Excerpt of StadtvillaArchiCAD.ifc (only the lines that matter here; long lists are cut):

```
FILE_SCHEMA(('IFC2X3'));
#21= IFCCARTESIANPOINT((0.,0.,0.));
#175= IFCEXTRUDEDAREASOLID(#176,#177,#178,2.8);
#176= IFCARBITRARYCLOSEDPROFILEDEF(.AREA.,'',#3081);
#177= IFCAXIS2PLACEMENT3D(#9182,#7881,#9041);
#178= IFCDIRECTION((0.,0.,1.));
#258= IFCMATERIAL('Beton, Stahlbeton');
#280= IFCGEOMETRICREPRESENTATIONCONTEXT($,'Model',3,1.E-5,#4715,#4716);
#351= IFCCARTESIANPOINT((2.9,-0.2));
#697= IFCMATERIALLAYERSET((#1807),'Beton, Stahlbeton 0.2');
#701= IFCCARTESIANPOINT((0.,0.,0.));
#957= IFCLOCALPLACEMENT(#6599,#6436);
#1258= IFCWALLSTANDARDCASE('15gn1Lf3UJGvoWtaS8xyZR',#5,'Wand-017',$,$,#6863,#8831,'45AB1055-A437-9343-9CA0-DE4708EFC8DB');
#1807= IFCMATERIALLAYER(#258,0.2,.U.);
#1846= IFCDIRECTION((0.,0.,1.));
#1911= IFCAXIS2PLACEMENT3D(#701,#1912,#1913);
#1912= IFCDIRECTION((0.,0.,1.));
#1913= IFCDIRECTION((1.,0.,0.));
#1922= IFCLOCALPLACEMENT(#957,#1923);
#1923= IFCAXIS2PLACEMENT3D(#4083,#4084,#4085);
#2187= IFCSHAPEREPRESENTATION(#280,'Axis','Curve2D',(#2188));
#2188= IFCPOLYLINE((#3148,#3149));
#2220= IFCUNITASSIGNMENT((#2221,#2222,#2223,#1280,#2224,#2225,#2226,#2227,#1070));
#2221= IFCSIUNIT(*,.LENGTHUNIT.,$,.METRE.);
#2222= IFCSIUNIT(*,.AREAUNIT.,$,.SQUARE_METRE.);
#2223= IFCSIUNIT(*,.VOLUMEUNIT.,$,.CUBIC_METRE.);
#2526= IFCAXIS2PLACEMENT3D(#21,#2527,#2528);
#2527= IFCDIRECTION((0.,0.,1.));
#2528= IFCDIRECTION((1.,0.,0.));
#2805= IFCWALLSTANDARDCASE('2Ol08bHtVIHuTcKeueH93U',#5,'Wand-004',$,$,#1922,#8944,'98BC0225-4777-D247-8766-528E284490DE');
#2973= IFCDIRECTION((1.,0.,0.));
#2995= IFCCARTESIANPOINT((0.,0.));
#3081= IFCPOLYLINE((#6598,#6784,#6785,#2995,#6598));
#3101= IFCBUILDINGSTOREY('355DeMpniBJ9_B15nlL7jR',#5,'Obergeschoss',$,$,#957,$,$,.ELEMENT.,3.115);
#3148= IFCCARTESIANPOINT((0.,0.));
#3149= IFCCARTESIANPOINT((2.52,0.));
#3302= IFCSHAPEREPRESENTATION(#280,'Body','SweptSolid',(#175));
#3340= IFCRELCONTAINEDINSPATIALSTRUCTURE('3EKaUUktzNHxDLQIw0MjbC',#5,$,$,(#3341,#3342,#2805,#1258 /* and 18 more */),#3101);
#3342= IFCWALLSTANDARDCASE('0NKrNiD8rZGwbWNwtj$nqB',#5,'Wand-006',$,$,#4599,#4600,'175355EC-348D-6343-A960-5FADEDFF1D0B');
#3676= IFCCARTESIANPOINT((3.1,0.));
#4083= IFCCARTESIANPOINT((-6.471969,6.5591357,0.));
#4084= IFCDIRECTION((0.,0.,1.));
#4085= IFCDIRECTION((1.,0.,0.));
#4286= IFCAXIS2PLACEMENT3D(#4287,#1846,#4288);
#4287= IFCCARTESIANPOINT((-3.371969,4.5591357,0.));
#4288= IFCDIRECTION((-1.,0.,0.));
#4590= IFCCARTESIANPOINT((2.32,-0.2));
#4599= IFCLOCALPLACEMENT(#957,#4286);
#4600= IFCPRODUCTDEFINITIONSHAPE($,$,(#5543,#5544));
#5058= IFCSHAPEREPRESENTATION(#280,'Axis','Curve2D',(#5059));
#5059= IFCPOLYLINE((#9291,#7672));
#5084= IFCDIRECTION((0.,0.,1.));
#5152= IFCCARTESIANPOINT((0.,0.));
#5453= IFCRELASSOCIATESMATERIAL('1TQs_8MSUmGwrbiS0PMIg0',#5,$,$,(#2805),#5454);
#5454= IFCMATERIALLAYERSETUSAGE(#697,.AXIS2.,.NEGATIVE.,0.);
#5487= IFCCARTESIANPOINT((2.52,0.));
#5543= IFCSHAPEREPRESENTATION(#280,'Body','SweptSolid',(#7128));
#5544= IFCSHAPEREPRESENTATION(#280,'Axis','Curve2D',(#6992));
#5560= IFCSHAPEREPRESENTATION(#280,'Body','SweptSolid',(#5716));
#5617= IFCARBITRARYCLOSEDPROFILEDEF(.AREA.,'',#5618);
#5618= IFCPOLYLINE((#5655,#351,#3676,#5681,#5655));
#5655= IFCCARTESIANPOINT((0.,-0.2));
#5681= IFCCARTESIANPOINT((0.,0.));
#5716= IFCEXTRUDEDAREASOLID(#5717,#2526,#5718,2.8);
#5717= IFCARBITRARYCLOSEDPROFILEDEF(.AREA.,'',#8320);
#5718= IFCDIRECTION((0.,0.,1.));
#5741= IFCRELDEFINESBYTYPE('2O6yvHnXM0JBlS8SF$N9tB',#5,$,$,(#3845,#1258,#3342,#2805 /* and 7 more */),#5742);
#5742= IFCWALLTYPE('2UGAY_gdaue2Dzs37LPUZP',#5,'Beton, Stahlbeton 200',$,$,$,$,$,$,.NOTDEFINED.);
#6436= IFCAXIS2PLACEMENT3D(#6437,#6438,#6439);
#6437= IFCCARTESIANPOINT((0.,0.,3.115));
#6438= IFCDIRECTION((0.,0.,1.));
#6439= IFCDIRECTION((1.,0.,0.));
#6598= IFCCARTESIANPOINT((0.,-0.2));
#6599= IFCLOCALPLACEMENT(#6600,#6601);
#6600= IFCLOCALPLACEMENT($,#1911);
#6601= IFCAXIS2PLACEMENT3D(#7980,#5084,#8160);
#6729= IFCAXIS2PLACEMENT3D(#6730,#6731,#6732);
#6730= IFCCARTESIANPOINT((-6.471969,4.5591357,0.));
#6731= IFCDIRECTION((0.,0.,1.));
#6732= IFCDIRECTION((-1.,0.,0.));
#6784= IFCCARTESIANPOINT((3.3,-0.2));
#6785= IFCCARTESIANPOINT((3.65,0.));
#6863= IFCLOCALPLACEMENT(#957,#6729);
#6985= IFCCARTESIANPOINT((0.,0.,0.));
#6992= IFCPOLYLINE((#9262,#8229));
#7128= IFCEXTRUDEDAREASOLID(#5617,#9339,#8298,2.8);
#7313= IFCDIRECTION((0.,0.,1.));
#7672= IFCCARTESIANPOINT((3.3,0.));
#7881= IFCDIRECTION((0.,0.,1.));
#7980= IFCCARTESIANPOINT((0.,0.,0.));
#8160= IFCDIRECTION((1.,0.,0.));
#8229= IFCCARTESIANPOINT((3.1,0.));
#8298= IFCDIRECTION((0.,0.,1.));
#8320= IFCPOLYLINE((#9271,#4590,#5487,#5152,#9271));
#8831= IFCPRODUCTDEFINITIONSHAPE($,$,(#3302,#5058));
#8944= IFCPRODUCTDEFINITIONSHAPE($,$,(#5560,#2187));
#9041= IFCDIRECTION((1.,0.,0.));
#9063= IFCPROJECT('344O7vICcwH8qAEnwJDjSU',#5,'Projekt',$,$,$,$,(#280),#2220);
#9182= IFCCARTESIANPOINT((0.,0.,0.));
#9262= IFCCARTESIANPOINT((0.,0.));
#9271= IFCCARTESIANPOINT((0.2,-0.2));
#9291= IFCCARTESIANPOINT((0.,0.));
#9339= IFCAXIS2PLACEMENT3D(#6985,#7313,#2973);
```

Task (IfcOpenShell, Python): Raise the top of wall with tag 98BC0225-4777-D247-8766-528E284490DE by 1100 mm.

```python
import ifcopenshell
import ifcopenshell.geom
import ifcopenshell.util.shape

model = ifcopenshell.open("StadtvillaArchiCAD.ifc")
settings = ifcopenshell.geom.settings()


def volume(element):
    """Net volume in cubic metres, openings subtracted."""
    shape = ifcopenshell.geom.create_shape(settings, element)
    return ifcopenshell.util.shape.get_volume(shape.geometry)


wall = model.by_id(2805)
before = volume(wall)

body = next(r for r in wall.Representation.Representations if r.RepresentationIdentifier == "Body")
solid = body.Items[0]
old_height = solid.Depth
solid.Depth += 1.1
after = volume(wall)

print(f"height {old_height:g} -> {solid.Depth:g}, volume {before:.3f} -> {after:.3f} m3")

model.write("StadtvillaArchiCAD_v2.ifc")
```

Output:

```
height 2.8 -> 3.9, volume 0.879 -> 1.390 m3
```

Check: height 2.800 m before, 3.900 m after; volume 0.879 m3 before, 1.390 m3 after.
